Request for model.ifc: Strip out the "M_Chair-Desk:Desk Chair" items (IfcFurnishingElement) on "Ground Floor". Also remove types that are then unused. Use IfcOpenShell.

First a look at what the model holds.

```python
import ifcopenshell
import ifcopenshell.util.element

model = ifcopenshell.open("model.ifc")
print(model.schema)
storey = next(s for s in model.by_type("IfcBuildingStorey") if s.Name == "Ground Floor")
furniture = [e for e in ifcopenshell.util.element.get_decomposition(storey) if e.is_a("IfcFurnishingElement")]
seen = {}
for e in furniture:
    element_type = ifcopenshell.util.element.get_type(e)
    name = element_type.Name if element_type not in (None, e) else None
    seen[name] = seen.get(name, 0) + 1
for name, count in sorted(seen.items(), key=str):
    print(count, "x", name)
```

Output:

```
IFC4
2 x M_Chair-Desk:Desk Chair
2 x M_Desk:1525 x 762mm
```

```python
import ifcopenshell
import ifcopenshell.api.root
import ifcopenshell.util.element

model = ifcopenshell.open("model.ifc")

storey = next(s for s in model.by_type("IfcBuildingStorey") if s.Name == "Ground Floor")
furniture = [e for e in ifcopenshell.util.element.get_decomposition(storey) if e.is_a("IfcFurnishingElement")]
targets = [e for e in furniture if (t := ifcopenshell.util.element.get_type(e)) not in (None, e) and t.Name == "M_Chair-Desk:Desk Chair"]
types = {ifcopenshell.util.element.get_type(e) for e in targets} - {None, *targets}

for e in targets:
    ifcopenshell.api.root.remove_product(model, product=e)
print(len(targets), "removed")

unused = [t for t in types if not ifcopenshell.util.element.get_types(t)]
for t in unused:
    ifcopenshell.api.root.remove_product(model, product=t)
print(len(unused), "unused types removed")

model.write("model_edited.ifc")
```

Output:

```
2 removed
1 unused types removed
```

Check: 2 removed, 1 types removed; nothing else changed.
